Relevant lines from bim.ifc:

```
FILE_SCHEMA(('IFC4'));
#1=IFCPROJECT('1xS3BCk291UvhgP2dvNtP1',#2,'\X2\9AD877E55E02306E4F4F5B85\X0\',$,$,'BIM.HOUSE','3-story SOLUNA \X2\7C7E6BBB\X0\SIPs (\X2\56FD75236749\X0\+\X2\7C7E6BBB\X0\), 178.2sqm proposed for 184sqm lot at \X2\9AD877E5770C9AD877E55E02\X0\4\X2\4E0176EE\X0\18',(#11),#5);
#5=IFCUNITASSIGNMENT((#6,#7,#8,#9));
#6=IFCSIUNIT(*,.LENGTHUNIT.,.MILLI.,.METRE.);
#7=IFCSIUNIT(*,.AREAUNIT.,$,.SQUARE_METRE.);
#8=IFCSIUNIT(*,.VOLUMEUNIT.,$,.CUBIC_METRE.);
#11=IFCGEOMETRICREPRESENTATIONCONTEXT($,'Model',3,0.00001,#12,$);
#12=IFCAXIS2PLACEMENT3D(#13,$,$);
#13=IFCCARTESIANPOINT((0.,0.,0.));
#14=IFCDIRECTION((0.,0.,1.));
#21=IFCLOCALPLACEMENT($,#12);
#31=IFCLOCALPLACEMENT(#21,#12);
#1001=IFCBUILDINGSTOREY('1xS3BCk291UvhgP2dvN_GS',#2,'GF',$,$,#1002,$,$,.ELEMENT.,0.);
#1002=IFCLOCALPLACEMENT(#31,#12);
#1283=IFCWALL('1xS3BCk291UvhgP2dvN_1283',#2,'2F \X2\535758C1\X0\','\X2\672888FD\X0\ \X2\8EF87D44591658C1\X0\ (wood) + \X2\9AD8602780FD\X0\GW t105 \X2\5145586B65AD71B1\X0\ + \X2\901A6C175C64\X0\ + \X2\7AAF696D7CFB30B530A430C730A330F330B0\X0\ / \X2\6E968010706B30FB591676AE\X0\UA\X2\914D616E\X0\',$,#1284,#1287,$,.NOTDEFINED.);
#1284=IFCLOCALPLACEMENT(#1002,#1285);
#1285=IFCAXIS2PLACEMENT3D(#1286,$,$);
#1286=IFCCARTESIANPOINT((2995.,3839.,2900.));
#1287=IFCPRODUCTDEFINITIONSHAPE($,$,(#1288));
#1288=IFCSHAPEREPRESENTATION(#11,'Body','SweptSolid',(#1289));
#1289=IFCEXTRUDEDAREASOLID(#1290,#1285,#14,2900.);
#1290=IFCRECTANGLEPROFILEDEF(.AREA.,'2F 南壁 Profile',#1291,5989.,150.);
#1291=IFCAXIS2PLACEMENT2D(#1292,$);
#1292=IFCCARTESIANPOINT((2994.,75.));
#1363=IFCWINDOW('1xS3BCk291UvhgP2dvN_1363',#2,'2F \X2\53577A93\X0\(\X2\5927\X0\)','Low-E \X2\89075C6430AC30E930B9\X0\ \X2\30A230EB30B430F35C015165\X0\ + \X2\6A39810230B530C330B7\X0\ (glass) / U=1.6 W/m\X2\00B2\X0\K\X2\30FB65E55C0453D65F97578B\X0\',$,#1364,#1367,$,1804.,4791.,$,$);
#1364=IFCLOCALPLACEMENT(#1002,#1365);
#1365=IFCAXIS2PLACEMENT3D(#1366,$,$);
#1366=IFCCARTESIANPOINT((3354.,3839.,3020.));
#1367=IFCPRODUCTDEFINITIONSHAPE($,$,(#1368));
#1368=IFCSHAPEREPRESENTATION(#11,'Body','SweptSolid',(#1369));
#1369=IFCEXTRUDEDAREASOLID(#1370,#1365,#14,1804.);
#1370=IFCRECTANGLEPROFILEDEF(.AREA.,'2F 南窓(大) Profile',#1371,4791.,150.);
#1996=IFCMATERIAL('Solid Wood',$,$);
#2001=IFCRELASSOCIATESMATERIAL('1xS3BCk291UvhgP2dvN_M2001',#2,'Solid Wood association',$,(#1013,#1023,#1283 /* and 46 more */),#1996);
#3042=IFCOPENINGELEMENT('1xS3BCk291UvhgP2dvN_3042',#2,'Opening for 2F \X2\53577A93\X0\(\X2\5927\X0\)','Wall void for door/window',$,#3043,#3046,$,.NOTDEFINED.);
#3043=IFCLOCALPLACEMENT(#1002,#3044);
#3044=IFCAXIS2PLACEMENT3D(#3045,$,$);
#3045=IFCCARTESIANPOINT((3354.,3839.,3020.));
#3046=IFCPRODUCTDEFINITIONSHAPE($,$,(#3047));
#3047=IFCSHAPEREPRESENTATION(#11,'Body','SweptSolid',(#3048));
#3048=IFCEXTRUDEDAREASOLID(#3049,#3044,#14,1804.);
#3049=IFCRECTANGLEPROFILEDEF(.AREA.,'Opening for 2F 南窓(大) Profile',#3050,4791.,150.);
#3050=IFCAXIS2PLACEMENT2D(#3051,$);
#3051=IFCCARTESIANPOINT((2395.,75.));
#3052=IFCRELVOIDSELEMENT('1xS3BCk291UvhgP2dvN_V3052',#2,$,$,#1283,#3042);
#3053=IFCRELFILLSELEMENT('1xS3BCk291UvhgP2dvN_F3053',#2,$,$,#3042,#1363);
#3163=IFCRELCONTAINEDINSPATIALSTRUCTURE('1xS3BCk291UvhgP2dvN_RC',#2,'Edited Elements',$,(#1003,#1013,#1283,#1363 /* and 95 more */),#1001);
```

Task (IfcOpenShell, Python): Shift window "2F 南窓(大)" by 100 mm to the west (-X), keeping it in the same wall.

```python
import ifcopenshell
import ifcopenshell.api.geometry
import ifcopenshell.util.placement
import ifcopenshell.util.unit

model = ifcopenshell.open("bim.ifc")
unit_scale = ifcopenshell.util.unit.calculate_unit_scale(model)

window = model.by_id(1363)
opening = window.FillsVoids[0].RelatingOpeningElement
wall = opening.VoidsElements[0].RelatingBuildingElement

wall_matrix = ifcopenshell.util.placement.get_local_placement(wall.ObjectPlacement)
shift = wall_matrix[:3, 0] * -0.1 / unit_scale
before = ifcopenshell.util.placement.get_local_placement(window.ObjectPlacement)[:3, 3].copy()

# The window is not placed relative to its opening, so move both.
for product in (opening, window):
    matrix = ifcopenshell.util.placement.get_local_placement(product.ObjectPlacement)
    matrix[:3, 3] += shift
    ifcopenshell.api.geometry.edit_object_placement(model, product=product, matrix=matrix, is_si=False)

after = ifcopenshell.util.placement.get_local_placement(window.ObjectPlacement)[:3, 3]
print("window moved by", (after - before).round(3) + 0.0)

model.write("bim-out.ifc")
```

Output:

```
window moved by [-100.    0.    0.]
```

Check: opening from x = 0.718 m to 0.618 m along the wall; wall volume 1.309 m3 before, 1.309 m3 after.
